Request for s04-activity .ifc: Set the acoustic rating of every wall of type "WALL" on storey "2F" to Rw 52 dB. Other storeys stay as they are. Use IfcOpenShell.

First a look at what the model holds.

```python
import ifcopenshell
import ifcopenshell.util.element

model = ifcopenshell.open("s04-activity .ifc")
print(model.schema)
storey = next(s for s in model.by_type("IfcBuildingStorey") if s.Name == "2F")
walls = [e for e in ifcopenshell.util.element.get_decomposition(storey) if e.is_a("IfcWall")]
seen = {}
for e in walls:
    element_type = ifcopenshell.util.element.get_type(e)
    key = (element_type.Name if element_type != e and element_type else None, ifcopenshell.util.element.get_pset(e, "Pset_WallCommon", "AcousticRating"))
    seen[key] = seen.get(key, 0) + 1
for (name, value), count in sorted(seen.items(), key=str):
    print(count, "x", name, "|", value)
```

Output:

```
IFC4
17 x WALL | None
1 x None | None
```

```python
import ifcopenshell
import ifcopenshell.api.pset
import ifcopenshell.util.element

model = ifcopenshell.open("s04-activity .ifc")

storey = next(s for s in model.by_type("IfcBuildingStorey") if s.Name == "2F")
walls = [e for e in ifcopenshell.util.element.get_decomposition(storey) if e.is_a("IfcWall")]

count = 0
for e in walls:
    element_type = ifcopenshell.util.element.get_type(e)
    if element_type in (None, e) or element_type.Name != "WALL":
        continue
    # add_pset returns the element's existing set when there is one.
    pset = ifcopenshell.api.pset.add_pset(model, product=e, name="Pset_WallCommon")
    ifcopenshell.api.pset.edit_pset(model, pset=pset, properties={"AcousticRating": "Rw 52 dB"})
    count += 1

print(count, "walls updated")

model.write("s04-activity -out.ifc")
```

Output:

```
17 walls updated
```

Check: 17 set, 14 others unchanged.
